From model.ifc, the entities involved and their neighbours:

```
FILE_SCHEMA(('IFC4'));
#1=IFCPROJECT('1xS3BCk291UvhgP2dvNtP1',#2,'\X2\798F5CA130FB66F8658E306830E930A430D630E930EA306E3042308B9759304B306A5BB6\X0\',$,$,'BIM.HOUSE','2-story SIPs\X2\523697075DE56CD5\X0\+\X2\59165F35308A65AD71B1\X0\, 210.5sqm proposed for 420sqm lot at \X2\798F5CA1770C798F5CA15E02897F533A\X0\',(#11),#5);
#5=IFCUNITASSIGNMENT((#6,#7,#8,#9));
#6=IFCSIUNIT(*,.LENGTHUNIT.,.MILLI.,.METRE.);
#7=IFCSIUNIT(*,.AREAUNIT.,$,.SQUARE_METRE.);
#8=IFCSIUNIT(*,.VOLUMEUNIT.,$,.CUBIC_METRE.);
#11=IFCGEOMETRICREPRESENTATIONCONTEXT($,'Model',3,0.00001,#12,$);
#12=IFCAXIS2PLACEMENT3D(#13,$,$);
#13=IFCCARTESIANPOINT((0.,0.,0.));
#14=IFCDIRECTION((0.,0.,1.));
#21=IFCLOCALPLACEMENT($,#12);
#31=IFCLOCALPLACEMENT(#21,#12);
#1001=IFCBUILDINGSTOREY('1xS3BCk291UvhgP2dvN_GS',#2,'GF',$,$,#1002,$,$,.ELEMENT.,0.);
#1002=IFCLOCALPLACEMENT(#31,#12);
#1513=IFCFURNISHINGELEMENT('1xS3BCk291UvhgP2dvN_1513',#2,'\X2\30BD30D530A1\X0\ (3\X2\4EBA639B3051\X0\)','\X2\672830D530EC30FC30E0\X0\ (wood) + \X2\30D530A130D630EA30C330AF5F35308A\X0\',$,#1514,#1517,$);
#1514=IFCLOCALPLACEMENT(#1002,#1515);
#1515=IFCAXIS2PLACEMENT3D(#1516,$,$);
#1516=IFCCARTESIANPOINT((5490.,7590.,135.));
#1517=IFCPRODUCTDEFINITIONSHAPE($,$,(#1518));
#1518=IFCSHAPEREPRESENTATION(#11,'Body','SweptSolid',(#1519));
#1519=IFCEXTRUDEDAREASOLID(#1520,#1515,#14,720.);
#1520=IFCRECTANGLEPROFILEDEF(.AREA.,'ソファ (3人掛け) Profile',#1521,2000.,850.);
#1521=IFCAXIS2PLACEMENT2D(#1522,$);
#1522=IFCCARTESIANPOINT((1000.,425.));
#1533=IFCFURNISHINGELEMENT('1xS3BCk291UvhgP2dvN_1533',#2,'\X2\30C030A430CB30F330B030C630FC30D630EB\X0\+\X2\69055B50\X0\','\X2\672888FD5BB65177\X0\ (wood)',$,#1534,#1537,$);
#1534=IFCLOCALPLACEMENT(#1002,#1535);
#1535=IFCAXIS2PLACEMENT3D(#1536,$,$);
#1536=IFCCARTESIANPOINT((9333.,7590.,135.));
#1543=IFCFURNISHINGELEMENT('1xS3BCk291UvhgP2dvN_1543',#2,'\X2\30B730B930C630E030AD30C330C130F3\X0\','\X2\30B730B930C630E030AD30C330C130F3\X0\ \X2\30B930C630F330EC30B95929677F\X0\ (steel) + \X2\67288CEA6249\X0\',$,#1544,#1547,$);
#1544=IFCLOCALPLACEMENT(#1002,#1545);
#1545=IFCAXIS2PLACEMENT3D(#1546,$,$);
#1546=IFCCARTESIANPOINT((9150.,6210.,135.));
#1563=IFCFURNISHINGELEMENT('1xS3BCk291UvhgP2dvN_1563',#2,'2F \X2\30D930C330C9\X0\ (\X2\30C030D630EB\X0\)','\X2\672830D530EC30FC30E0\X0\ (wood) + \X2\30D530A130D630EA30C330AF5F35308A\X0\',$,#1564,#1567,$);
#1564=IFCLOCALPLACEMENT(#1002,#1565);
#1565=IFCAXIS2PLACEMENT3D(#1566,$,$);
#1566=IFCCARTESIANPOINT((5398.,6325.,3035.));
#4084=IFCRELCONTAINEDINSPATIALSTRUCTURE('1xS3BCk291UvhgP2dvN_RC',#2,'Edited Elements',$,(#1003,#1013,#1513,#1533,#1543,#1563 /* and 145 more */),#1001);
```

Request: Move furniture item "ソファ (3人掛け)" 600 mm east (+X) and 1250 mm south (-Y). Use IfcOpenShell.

```python
import ifcopenshell
import ifcopenshell.api.geometry
import ifcopenshell.util.placement
import ifcopenshell.util.unit

model = ifcopenshell.open("model.ifc")
unit_scale = ifcopenshell.util.unit.calculate_unit_scale(model)

item = model.by_id(1513)
matrix = ifcopenshell.util.placement.get_local_placement(item.ObjectPlacement)
matrix[0, 3] += 0.6 / unit_scale
matrix[1, 3] -= 1.25 / unit_scale
ifcopenshell.api.geometry.edit_object_placement(model, product=item, matrix=matrix, is_si=False)

print(ifcopenshell.util.placement.get_local_placement(item.ObjectPlacement).round(3) + 0.0)

model.write("model_edited.ifc")
```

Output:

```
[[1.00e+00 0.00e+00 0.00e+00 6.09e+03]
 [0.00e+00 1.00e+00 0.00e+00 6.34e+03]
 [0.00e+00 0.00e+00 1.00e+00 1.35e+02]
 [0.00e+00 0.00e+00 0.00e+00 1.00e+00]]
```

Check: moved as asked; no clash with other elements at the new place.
